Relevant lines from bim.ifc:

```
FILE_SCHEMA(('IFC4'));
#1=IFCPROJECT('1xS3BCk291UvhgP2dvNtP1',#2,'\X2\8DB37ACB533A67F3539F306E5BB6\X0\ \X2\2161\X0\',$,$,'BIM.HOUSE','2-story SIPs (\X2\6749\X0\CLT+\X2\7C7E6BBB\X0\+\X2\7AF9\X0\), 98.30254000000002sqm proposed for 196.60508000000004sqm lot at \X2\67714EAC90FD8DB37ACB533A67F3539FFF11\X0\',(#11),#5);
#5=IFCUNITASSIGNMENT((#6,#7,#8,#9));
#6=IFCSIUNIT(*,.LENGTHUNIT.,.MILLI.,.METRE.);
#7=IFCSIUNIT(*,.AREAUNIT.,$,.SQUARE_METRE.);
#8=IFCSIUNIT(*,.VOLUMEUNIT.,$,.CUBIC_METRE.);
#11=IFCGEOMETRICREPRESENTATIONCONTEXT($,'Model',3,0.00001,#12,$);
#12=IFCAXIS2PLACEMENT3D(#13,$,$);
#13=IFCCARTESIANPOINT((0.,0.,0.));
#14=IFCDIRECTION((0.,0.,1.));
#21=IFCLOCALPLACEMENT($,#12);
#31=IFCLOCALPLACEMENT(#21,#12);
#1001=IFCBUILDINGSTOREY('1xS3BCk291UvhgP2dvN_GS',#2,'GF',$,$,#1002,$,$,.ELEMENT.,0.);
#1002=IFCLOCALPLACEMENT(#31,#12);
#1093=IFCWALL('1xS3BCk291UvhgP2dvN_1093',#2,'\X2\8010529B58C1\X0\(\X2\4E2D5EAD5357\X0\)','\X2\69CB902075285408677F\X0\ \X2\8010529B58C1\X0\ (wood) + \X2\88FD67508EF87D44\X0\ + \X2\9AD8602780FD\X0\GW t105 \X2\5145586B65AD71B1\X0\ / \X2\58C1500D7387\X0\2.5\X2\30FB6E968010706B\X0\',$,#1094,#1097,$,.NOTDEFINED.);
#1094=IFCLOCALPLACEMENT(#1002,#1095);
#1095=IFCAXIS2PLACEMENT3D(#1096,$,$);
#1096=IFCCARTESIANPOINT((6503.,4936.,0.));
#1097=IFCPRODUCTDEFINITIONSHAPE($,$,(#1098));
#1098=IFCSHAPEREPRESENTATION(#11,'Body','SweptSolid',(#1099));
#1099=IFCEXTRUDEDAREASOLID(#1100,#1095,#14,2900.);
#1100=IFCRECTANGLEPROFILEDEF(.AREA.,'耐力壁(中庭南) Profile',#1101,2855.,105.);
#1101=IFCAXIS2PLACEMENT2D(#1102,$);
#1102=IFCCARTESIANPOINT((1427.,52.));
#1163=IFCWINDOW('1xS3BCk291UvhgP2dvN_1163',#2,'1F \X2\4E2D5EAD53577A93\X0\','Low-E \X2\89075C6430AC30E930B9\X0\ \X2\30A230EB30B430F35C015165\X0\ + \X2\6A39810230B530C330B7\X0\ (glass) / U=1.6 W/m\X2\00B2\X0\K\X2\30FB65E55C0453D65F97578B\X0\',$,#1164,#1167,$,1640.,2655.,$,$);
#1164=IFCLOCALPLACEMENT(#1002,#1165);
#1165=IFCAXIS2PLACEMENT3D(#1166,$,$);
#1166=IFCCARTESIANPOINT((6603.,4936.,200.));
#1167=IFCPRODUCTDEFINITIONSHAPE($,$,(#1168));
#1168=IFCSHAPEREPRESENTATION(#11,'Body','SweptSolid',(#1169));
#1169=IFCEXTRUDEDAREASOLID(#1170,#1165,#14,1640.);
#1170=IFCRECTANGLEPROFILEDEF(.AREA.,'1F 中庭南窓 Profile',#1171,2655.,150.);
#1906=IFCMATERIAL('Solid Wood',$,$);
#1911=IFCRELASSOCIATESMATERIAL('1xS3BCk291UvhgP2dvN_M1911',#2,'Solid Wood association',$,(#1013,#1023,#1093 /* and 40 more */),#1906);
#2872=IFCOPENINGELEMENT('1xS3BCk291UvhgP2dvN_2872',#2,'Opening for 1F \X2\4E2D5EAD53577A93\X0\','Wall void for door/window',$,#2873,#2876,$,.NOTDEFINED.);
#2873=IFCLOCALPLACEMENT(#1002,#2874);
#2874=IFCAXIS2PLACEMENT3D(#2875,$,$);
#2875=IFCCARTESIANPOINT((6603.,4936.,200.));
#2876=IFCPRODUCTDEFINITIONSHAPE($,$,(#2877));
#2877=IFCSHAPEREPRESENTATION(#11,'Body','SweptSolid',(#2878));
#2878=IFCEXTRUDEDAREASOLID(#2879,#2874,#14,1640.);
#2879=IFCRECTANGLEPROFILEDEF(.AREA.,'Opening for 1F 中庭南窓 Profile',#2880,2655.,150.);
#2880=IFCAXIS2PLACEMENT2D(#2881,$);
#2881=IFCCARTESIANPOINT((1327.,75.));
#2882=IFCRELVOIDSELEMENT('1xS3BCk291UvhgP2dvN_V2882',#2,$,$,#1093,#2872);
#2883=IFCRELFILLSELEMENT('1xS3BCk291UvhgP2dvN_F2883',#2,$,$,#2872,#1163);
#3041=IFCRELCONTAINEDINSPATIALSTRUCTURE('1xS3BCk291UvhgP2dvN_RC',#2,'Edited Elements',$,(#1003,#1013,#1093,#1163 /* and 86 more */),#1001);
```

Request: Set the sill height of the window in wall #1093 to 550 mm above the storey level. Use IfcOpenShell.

```python
import numpy as np
import ifcopenshell
import ifcopenshell.api.geometry
import ifcopenshell.geom
import ifcopenshell.util.element
import ifcopenshell.util.placement
import ifcopenshell.util.shape
import ifcopenshell.util.unit

model = ifcopenshell.open("bim.ifc")
unit_scale = ifcopenshell.util.unit.calculate_unit_scale(model)

window = model.by_guid("1xS3BCk291UvhgP2dvN_1163")
opening = window.FillsVoids[0].RelatingOpeningElement
storey = ifcopenshell.util.element.get_container(window, ifc_class="IfcBuildingStorey")
level = ifcopenshell.util.placement.get_local_placement(storey.ObjectPlacement)[2, 3]

# The opening's origin need not be at the sill, so measure its lowest point.
shape = ifcopenshell.geom.create_shape(ifcopenshell.geom.settings(), opening)
bottom = ifcopenshell.util.shape.get_shape_bottom_elevation(shape, shape.geometry) / unit_scale
dz = level + 0.55 / unit_scale - bottom

shift = np.array([0.0, 0.0, dz])
# The window is not placed relative to its opening, so move both.
for product in (opening, window):
    matrix = ifcopenshell.util.placement.get_local_placement(product.ObjectPlacement)
    matrix[:3, 3] += shift
    ifcopenshell.api.geometry.edit_object_placement(model, product=product, matrix=matrix, is_si=False)

print(f"moved by {dz * unit_scale:+.3f} m")

model.write("bim-out.ifc")
```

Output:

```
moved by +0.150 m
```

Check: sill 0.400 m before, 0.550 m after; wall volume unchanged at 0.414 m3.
